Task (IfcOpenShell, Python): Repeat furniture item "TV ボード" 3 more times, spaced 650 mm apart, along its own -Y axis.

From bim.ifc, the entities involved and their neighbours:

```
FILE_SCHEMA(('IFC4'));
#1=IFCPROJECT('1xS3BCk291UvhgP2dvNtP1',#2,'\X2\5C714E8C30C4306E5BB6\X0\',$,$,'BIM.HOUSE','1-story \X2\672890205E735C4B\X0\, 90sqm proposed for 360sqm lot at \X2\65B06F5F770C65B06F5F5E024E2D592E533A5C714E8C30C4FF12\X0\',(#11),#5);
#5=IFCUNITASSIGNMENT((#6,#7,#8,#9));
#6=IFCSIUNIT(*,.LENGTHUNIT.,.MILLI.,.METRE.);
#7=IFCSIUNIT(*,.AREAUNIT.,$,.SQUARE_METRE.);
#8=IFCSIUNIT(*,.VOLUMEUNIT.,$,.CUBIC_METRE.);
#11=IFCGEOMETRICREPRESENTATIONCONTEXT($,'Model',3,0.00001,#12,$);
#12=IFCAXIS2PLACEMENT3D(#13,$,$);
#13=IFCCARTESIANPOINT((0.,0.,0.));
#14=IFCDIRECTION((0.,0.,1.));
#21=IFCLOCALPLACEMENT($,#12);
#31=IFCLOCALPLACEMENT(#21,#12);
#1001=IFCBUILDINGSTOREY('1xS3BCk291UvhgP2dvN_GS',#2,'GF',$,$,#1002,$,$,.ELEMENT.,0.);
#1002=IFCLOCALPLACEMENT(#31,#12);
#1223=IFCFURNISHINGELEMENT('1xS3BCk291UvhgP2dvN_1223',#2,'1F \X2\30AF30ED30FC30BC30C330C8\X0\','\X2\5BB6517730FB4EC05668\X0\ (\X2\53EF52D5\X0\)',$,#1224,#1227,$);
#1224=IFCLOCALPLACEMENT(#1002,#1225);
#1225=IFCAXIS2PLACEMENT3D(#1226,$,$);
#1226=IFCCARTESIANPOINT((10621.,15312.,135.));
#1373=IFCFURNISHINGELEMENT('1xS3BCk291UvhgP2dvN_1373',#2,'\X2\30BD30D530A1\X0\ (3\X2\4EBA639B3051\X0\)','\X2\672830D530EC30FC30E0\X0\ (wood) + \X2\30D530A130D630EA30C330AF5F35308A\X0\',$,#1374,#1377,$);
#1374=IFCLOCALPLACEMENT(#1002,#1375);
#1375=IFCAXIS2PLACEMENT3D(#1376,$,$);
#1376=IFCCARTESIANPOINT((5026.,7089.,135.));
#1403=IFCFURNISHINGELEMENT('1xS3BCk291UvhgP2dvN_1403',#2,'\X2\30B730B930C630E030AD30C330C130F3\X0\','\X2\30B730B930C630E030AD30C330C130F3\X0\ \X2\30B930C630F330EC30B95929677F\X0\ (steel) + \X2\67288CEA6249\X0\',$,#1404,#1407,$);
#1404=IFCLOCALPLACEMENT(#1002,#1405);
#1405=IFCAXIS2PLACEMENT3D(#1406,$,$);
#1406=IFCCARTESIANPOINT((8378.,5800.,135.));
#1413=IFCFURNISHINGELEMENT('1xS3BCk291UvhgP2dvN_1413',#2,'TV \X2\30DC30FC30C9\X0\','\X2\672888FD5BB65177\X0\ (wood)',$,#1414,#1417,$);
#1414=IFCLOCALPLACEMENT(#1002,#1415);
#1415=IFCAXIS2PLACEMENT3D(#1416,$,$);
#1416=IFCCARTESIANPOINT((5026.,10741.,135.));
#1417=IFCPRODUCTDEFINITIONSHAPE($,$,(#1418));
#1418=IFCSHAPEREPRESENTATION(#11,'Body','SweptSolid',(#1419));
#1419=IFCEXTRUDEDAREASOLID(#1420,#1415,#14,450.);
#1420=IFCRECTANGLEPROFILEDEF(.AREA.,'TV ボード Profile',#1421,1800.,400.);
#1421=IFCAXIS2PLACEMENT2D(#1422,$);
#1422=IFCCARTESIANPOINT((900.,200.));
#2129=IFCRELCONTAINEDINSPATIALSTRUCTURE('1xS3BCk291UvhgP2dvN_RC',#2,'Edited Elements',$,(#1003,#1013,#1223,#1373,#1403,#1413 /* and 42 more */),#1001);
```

```python
import ifcopenshell
import ifcopenshell.api.geometry
import ifcopenshell.api.root
import ifcopenshell.util.element
import ifcopenshell.util.placement
import ifcopenshell.util.unit

model = ifcopenshell.open("bim.ifc")
unit_scale = ifcopenshell.util.unit.calculate_unit_scale(model)


def reuse_history(source, copy):
    """copy_class also copies each property set's owner history, people and application; keep the originals."""
    for rel in copy.IsDefinedBy:
        if rel.is_a("IfcRelDefinesByProperties") and (history := rel.RelatingPropertyDefinition.OwnerHistory):
            rel.RelatingPropertyDefinition.OwnerHistory = source.OwnerHistory
            ifcopenshell.util.element.remove_deep2(model, history)


source = model.by_guid("1xS3BCk291UvhgP2dvN_1413")
base = ifcopenshell.util.placement.get_local_placement(source.ObjectPlacement)
step = -base[:3, 1] * 0.65 / unit_scale

for i in range(1, 4):
    copy = ifcopenshell.api.root.copy_class(model, product=source)
    copy.Representation = ifcopenshell.util.element.copy_deep(
        model, source.Representation, exclude=["IfcGeometricRepresentationContext", "IfcRepresentationMap"]
    )
    reuse_history(source, copy)
    matrix = base.copy()
    matrix[:3, 3] += i * step
    print("added at", matrix[:3, 3].round(3) + 0.0)
    ifcopenshell.api.geometry.edit_object_placement(model, product=copy, matrix=matrix, is_si=False)

model.write("bim_edited.ifc")
```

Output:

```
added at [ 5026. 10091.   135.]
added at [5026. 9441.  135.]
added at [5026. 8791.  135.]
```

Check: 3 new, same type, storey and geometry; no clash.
